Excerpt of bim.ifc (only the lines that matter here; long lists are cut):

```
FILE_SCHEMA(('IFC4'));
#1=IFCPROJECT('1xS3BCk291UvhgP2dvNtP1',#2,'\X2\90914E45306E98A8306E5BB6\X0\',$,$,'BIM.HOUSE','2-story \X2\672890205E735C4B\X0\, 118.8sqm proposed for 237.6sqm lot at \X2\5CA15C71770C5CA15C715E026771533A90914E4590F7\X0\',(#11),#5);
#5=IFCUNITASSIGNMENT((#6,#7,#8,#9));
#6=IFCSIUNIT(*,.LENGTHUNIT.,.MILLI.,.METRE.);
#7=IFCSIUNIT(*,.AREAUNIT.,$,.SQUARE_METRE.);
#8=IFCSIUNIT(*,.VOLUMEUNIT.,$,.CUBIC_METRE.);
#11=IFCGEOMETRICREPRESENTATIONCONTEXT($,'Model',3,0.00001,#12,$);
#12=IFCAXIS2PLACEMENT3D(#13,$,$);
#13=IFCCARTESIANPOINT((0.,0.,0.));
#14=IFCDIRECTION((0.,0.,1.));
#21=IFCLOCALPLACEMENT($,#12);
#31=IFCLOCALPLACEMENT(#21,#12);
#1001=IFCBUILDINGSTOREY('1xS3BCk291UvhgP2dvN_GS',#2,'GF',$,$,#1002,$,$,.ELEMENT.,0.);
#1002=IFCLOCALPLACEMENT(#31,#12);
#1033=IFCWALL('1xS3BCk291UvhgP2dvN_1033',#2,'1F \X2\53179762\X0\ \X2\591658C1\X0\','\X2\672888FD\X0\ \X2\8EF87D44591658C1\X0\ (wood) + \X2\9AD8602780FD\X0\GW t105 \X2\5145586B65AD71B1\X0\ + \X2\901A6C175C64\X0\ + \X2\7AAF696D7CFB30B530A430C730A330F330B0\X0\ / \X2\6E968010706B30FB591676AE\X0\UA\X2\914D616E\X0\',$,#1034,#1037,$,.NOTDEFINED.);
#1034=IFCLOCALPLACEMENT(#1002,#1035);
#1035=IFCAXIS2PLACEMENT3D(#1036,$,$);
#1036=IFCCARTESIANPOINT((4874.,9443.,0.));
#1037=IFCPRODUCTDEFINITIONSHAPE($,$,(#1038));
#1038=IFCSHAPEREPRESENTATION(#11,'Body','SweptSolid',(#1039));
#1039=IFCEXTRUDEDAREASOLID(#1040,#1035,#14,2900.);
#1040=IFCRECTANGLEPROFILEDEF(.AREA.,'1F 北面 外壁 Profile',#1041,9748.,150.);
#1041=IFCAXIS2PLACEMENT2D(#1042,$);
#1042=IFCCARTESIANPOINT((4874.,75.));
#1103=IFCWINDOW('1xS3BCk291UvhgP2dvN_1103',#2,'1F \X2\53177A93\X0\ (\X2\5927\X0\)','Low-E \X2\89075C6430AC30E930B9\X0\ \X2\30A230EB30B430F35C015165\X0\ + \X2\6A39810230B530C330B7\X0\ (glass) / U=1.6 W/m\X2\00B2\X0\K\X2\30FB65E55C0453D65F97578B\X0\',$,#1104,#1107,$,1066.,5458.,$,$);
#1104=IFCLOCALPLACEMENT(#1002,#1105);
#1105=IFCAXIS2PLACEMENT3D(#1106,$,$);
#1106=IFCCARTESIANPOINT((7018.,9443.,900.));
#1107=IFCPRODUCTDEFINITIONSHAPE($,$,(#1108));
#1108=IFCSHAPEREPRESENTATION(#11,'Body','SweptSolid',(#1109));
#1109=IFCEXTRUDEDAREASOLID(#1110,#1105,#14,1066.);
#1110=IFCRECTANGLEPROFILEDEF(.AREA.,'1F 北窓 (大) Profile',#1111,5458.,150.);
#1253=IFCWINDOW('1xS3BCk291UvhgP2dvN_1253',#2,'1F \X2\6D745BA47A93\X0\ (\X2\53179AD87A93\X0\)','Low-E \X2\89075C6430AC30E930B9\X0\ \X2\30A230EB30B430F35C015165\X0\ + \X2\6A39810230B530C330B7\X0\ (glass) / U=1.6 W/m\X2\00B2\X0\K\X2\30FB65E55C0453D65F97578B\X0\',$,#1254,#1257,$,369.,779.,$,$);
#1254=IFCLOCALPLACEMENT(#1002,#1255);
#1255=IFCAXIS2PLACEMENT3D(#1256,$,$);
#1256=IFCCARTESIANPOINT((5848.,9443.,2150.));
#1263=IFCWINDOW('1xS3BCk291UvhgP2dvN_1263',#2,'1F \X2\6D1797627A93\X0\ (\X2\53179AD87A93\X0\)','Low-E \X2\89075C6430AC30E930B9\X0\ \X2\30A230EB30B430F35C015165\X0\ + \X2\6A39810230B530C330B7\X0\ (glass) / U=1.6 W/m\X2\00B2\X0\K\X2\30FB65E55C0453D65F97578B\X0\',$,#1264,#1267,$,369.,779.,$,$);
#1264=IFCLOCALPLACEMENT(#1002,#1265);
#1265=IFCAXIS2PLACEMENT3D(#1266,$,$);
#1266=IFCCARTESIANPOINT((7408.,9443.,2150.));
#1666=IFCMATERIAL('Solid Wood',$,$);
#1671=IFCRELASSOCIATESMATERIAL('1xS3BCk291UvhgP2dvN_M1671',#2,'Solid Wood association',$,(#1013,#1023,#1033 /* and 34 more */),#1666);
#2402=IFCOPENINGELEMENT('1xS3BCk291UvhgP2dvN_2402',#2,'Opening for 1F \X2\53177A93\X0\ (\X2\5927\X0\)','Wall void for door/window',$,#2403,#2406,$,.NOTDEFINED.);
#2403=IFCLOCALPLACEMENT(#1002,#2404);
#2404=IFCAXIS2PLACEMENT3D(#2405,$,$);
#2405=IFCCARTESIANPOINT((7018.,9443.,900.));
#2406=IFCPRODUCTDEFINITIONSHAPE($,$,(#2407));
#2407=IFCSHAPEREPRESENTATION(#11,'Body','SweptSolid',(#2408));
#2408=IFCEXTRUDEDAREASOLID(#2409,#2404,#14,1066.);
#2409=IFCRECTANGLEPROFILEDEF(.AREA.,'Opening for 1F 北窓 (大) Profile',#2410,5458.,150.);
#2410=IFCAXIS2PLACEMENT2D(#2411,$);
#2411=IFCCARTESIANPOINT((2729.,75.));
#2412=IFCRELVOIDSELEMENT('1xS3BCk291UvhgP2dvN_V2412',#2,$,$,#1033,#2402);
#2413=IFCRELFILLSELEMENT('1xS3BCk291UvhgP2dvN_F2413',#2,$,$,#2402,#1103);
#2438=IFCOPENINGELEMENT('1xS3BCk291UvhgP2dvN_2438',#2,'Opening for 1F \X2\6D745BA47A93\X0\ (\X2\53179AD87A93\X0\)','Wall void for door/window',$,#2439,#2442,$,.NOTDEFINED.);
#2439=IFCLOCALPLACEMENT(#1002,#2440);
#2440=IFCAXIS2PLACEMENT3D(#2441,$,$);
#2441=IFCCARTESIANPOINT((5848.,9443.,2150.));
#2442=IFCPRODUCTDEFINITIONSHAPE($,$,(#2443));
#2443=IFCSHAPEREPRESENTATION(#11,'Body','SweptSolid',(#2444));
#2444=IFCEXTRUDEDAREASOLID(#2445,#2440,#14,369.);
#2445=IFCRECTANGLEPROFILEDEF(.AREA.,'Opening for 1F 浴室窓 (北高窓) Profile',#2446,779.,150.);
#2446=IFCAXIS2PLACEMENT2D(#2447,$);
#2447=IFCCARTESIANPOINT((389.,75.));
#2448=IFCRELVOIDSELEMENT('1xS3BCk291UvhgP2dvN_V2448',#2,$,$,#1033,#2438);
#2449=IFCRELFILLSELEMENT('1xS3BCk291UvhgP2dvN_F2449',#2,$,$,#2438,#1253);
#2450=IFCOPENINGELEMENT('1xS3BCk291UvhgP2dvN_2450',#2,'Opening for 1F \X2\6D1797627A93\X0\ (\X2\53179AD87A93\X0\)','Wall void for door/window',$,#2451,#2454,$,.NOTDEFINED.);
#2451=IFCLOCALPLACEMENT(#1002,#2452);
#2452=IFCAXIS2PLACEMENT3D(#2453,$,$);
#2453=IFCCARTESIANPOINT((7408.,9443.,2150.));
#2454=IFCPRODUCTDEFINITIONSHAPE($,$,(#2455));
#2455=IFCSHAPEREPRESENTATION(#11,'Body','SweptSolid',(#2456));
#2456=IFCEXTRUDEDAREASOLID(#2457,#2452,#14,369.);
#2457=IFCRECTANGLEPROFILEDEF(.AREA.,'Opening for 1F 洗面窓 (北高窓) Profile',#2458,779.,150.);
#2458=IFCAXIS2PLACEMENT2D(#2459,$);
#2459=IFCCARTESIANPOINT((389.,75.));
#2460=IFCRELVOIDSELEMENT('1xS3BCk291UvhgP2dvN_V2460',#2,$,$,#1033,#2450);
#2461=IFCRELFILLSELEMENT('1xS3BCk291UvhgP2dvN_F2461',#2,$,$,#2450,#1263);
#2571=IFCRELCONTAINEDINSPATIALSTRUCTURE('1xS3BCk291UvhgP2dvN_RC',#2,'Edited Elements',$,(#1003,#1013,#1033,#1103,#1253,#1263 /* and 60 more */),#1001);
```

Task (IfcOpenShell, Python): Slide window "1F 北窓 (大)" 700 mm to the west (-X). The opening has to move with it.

```python
import ifcopenshell
import ifcopenshell.api.geometry
import ifcopenshell.util.placement

model = ifcopenshell.open("bim.ifc")

window = model.by_guid("1xS3BCk291UvhgP2dvN_1103")
opening = window.FillsVoids[0].RelatingOpeningElement
wall = opening.VoidsElements[0].RelatingBuildingElement

wall_matrix = ifcopenshell.util.placement.get_local_placement(wall.ObjectPlacement)
shift = wall_matrix[:3, 0] * -700.0
before = ifcopenshell.util.placement.get_local_placement(window.ObjectPlacement)[:3, 3].copy()

# The window is not placed relative to its opening, so move both.
for product in (opening, window):
    matrix = ifcopenshell.util.placement.get_local_placement(product.ObjectPlacement)
    matrix[:3, 3] += shift
    ifcopenshell.api.geometry.edit_object_placement(model, product=product, matrix=matrix, is_si=False)

after = ifcopenshell.util.placement.get_local_placement(window.ObjectPlacement)[:3, 3]
print("window moved by", (after - before).round(3) + 0.0)

model.write("bim_rev.ifc")
```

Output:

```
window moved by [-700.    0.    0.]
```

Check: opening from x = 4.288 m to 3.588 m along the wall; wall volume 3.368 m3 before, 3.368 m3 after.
